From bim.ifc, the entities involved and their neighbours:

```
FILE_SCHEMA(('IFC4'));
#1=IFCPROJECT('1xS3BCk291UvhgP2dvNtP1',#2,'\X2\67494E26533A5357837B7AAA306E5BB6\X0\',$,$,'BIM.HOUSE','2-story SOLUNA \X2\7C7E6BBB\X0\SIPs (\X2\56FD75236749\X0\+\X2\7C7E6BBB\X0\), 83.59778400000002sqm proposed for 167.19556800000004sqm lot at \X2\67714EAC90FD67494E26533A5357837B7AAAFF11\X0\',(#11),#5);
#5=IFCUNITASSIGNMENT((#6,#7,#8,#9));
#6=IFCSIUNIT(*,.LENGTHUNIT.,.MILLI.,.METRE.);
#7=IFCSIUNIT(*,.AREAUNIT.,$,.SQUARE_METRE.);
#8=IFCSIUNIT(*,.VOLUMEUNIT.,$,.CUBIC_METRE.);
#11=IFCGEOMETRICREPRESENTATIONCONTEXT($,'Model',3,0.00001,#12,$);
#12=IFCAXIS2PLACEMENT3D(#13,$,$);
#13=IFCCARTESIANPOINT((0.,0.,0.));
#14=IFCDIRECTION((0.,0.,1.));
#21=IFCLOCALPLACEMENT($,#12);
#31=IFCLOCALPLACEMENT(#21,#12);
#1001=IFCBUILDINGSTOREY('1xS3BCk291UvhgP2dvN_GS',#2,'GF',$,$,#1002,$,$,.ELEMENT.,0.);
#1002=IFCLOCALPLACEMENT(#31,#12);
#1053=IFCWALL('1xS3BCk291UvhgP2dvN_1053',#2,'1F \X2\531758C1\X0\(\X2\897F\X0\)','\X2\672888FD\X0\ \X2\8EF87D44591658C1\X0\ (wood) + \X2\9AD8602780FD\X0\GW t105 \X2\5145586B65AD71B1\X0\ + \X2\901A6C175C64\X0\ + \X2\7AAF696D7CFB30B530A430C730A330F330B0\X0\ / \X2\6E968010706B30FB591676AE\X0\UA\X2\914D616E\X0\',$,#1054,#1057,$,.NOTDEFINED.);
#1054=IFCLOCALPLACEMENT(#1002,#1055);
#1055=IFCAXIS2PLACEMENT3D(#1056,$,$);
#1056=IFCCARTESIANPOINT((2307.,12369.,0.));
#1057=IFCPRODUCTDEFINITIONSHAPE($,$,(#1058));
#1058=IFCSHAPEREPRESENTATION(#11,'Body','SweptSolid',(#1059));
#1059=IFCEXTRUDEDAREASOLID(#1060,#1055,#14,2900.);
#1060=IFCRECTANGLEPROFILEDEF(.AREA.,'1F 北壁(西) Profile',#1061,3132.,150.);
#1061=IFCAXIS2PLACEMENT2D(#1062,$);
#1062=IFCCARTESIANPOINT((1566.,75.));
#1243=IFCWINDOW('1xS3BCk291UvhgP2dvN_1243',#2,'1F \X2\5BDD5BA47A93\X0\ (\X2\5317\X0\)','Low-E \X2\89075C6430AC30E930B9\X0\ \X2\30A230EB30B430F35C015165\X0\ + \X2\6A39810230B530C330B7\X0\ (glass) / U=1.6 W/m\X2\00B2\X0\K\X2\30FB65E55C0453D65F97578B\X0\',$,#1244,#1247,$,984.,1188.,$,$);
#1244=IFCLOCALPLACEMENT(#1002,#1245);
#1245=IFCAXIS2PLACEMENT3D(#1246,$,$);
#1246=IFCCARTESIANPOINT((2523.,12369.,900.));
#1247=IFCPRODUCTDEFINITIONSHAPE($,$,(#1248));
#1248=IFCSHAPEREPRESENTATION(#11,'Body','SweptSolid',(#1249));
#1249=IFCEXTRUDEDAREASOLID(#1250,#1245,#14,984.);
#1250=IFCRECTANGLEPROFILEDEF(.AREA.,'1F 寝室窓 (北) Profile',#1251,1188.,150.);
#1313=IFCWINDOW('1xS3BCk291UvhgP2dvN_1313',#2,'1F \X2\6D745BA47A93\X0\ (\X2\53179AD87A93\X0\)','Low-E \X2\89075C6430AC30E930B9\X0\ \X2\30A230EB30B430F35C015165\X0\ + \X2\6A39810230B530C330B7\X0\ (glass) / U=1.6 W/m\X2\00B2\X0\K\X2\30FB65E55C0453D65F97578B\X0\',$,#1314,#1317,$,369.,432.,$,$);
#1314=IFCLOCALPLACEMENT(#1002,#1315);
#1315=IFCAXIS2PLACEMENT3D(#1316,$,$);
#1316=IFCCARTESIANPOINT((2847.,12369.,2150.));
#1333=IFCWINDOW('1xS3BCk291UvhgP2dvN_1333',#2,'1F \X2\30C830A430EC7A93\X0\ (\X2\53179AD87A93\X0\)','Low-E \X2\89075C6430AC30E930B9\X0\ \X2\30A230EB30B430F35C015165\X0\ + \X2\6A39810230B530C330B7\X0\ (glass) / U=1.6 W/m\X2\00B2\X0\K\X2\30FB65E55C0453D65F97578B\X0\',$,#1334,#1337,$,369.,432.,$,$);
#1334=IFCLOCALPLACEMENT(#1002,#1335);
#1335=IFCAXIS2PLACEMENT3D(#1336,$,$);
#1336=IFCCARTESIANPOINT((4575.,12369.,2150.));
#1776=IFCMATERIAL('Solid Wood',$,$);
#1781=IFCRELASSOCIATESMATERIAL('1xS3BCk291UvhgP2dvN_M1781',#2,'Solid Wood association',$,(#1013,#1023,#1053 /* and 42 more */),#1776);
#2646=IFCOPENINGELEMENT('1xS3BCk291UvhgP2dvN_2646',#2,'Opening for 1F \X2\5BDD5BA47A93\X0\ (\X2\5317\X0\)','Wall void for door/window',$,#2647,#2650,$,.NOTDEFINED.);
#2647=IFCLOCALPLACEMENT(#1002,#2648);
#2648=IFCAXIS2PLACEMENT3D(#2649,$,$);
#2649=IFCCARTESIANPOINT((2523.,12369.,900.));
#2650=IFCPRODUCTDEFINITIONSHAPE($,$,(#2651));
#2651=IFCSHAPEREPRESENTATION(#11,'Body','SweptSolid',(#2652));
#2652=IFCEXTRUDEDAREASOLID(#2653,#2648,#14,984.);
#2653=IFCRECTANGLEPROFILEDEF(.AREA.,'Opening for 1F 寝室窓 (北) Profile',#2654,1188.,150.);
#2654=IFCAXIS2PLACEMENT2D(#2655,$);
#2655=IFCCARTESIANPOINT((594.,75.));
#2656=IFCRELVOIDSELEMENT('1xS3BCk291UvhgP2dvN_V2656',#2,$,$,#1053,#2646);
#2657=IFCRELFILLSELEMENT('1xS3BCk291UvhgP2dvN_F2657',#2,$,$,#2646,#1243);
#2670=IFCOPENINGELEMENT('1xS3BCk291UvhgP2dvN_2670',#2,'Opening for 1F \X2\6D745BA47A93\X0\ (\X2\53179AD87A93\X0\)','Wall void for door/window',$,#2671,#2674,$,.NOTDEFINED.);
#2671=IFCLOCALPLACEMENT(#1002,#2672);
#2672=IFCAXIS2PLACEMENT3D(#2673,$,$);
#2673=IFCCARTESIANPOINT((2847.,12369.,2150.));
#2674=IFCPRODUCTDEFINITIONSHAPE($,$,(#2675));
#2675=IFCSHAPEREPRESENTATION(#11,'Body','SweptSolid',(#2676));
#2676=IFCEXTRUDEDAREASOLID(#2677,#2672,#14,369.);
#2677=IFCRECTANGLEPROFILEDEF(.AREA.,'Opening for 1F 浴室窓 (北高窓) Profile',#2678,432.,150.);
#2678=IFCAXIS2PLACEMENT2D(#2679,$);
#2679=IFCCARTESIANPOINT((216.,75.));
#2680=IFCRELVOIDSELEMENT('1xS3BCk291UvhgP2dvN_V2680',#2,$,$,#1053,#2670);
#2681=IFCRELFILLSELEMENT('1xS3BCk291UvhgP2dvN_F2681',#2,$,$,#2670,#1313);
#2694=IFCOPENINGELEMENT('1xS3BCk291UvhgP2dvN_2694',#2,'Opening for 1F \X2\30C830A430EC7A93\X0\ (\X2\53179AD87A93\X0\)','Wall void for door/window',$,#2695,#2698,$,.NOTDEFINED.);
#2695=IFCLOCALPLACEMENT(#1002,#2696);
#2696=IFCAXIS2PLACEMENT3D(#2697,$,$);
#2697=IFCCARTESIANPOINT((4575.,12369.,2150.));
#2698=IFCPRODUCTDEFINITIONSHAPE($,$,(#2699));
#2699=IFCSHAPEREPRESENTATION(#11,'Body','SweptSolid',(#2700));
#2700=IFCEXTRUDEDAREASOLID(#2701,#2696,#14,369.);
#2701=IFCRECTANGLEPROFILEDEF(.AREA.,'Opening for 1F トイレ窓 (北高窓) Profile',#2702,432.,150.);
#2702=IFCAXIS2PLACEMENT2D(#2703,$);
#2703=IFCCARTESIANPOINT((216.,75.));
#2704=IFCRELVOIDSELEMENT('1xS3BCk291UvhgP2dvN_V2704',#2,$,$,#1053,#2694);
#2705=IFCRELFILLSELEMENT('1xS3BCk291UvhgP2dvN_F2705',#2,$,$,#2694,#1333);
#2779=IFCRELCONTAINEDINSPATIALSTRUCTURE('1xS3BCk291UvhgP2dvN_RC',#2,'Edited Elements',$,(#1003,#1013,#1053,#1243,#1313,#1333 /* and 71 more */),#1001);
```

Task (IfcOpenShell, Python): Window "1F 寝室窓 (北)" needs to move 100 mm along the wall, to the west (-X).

```python
import ifcopenshell
import ifcopenshell.api.geometry
import ifcopenshell.util.placement

model = ifcopenshell.open("bim.ifc")

window = model.by_id(1243)
opening = window.FillsVoids[0].RelatingOpeningElement
wall = opening.VoidsElements[0].RelatingBuildingElement

wall_matrix = ifcopenshell.util.placement.get_local_placement(wall.ObjectPlacement)
shift = wall_matrix[:3, 0] * -100.0
before = ifcopenshell.util.placement.get_local_placement(window.ObjectPlacement)[:3, 3].copy()

# The window is not placed relative to its opening, so move both.
for product in (opening, window):
    matrix = ifcopenshell.util.placement.get_local_placement(product.ObjectPlacement)
    matrix[:3, 3] += shift
    ifcopenshell.api.geometry.edit_object_placement(model, product=product, matrix=matrix, is_si=False)

after = ifcopenshell.util.placement.get_local_placement(window.ObjectPlacement)[:3, 3]
print("window moved by", (after - before).round(3) + 0.0)

model.write("bim_edited.ifc")
```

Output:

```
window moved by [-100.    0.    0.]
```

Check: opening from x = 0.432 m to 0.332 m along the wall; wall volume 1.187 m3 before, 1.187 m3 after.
